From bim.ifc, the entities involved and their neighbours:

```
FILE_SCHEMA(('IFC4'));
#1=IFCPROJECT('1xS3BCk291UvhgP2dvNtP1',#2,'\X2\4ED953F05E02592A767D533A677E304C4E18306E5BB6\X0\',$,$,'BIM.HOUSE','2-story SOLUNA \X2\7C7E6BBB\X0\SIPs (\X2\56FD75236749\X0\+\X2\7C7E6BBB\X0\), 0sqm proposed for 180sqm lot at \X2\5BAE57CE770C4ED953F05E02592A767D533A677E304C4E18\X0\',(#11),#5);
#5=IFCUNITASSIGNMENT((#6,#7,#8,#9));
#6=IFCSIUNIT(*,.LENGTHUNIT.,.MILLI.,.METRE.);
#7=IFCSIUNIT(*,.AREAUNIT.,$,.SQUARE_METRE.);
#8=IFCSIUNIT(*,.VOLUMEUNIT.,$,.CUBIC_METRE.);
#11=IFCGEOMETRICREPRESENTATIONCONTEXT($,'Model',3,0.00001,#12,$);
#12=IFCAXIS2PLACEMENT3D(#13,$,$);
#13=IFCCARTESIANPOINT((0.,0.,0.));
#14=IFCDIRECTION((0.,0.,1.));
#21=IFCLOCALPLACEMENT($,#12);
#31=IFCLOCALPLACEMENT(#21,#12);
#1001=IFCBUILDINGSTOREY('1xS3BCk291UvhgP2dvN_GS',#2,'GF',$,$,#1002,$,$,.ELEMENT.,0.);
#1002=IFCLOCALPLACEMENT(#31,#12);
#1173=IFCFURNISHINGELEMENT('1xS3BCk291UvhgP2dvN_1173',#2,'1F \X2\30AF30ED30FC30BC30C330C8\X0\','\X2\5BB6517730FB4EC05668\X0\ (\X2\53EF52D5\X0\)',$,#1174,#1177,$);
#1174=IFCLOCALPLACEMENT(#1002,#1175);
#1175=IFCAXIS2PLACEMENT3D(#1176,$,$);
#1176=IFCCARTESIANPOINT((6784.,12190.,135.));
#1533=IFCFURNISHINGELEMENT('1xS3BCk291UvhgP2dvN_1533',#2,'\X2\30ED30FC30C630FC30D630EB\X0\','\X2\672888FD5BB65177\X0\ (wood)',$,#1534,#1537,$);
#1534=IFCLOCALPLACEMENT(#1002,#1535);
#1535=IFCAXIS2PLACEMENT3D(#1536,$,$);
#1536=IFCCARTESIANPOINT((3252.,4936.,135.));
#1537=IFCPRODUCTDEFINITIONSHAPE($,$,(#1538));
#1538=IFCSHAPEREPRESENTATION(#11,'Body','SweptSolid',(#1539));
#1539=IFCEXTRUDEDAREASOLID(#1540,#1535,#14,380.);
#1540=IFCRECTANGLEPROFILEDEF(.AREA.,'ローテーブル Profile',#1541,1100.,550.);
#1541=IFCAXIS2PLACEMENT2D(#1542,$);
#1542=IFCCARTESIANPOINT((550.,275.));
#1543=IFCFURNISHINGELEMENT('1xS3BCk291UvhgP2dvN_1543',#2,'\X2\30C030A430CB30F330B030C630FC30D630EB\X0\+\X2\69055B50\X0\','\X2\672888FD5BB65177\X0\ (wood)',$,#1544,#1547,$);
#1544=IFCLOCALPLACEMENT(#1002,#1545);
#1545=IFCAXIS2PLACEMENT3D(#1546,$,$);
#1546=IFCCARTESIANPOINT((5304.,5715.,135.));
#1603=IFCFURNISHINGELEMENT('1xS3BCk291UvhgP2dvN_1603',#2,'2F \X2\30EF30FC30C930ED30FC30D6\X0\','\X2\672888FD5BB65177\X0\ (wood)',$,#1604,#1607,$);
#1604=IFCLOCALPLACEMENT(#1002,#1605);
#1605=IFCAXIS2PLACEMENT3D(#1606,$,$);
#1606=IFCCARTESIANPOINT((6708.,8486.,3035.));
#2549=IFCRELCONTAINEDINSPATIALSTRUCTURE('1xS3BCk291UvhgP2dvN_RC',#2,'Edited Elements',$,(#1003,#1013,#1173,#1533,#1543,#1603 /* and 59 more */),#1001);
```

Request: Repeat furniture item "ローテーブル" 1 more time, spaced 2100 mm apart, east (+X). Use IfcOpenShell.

```python
import numpy as np
import ifcopenshell
import ifcopenshell.api.geometry
import ifcopenshell.api.root
import ifcopenshell.util.element
import ifcopenshell.util.placement
import ifcopenshell.util.unit

model = ifcopenshell.open("bim.ifc")
unit_scale = ifcopenshell.util.unit.calculate_unit_scale(model)


def reuse_history(source, copy):
    """copy_class also copies each property set's owner history, people and application; keep the originals."""
    for rel in copy.IsDefinedBy:
        if rel.is_a("IfcRelDefinesByProperties") and (history := rel.RelatingPropertyDefinition.OwnerHistory):
            rel.RelatingPropertyDefinition.OwnerHistory = source.OwnerHistory
            ifcopenshell.util.element.remove_deep2(model, history)


source = model.by_id(1533)
base = ifcopenshell.util.placement.get_local_placement(source.ObjectPlacement)
step = np.array([1.0, 0.0, 0.0]) * 2.1 / unit_scale

for i in range(1, 2):
    copy = ifcopenshell.api.root.copy_class(model, product=source)
    copy.Representation = ifcopenshell.util.element.copy_deep(
        model, source.Representation, exclude=["IfcGeometricRepresentationContext", "IfcRepresentationMap"]
    )
    reuse_history(source, copy)
    matrix = base.copy()
    matrix[:3, 3] += i * step
    print("added at", matrix[:3, 3].round(3) + 0.0)
    ifcopenshell.api.geometry.edit_object_placement(model, product=copy, matrix=matrix, is_si=False)

model.write("bim_edited.ifc")
```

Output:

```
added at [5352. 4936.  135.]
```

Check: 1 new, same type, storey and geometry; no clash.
